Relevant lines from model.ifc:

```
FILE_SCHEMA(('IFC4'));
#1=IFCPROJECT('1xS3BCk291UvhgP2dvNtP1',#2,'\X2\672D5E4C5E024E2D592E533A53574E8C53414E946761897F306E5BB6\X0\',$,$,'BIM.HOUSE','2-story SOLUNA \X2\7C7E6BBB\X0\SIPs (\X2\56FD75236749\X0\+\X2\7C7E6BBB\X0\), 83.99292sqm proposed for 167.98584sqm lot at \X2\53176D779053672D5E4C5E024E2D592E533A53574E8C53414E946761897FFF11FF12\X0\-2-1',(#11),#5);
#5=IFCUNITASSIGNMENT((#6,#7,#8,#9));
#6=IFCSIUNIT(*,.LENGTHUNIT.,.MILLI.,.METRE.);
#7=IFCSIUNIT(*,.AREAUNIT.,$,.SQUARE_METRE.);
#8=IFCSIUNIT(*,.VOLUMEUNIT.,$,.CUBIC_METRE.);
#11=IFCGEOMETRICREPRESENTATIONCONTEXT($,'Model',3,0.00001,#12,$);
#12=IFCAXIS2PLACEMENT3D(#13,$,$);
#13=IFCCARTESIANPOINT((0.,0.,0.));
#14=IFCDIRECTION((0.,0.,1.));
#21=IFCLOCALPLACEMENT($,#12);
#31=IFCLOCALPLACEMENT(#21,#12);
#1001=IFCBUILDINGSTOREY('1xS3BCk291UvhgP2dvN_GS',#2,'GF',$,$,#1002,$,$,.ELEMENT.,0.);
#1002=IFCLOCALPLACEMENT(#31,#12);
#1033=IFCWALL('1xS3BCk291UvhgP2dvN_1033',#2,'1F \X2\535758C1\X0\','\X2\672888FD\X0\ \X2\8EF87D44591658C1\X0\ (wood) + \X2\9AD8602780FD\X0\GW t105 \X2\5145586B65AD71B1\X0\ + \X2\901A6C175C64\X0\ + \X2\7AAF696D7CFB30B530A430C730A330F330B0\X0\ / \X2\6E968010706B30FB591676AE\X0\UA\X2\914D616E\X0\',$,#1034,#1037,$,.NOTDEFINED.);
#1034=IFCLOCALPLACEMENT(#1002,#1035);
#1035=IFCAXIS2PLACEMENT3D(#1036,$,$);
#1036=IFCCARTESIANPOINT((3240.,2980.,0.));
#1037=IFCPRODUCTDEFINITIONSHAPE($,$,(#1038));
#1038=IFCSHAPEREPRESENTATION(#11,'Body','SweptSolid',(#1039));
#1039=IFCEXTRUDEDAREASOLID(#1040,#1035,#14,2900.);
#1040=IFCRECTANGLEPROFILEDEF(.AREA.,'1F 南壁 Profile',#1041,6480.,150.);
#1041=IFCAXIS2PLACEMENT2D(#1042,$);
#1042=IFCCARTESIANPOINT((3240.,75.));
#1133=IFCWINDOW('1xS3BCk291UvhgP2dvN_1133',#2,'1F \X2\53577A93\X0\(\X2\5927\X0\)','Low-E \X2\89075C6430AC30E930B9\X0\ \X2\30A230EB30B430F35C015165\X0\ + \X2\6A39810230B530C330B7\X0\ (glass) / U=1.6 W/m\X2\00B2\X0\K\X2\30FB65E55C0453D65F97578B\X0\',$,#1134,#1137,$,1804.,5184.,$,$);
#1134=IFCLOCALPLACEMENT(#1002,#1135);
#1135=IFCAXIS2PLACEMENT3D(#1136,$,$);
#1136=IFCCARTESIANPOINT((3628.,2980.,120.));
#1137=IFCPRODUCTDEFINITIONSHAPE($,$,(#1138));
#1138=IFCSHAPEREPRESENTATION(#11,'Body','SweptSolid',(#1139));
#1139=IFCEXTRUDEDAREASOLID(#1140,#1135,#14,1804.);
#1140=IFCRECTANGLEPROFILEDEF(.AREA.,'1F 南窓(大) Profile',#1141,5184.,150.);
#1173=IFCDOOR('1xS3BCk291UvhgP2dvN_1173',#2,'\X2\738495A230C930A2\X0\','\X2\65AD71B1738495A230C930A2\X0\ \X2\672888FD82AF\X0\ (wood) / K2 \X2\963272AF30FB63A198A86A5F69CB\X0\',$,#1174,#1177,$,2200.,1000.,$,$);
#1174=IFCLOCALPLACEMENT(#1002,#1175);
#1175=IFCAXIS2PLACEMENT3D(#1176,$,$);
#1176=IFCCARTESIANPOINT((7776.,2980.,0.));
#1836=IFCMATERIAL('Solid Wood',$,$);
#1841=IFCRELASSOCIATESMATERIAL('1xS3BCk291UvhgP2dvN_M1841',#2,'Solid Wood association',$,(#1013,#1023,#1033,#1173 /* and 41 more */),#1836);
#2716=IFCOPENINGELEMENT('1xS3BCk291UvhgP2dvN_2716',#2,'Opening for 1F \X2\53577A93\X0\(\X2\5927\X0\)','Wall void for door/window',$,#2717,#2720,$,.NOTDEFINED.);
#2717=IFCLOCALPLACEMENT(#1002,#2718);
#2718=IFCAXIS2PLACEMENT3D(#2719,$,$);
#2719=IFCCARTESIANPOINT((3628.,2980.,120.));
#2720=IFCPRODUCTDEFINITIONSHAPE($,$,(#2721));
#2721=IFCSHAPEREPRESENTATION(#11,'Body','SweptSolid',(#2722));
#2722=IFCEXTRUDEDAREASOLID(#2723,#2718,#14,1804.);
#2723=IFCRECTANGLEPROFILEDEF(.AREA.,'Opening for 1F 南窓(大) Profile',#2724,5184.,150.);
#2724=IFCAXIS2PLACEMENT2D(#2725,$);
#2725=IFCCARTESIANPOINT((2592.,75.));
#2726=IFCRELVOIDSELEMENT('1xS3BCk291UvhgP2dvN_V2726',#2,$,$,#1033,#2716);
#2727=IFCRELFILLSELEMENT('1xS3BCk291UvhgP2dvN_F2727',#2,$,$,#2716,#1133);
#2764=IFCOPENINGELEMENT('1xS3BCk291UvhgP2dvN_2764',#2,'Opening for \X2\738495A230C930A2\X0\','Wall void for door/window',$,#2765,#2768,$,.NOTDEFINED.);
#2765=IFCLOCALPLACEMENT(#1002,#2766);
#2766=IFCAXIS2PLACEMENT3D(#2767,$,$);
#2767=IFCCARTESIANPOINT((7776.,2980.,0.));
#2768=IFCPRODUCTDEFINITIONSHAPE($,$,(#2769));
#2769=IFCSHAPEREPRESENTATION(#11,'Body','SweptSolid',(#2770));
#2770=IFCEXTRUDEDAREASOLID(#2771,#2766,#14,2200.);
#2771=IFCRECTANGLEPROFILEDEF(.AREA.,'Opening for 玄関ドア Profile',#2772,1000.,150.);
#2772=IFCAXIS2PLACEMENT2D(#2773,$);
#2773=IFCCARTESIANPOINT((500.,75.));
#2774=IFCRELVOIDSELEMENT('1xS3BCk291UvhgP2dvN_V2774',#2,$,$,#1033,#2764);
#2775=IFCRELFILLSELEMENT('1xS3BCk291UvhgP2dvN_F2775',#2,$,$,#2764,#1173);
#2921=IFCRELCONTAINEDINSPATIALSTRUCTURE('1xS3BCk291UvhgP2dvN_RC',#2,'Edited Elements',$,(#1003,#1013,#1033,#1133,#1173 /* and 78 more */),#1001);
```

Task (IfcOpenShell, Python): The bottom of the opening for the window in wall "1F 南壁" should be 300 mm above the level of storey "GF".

```python
import numpy as np
import ifcopenshell
import ifcopenshell.api.geometry
import ifcopenshell.geom
import ifcopenshell.util.element
import ifcopenshell.util.placement
import ifcopenshell.util.shape
import ifcopenshell.util.unit

model = ifcopenshell.open("model.ifc")
unit_scale = ifcopenshell.util.unit.calculate_unit_scale(model)

window = model.by_guid("1xS3BCk291UvhgP2dvN_1133")
opening = window.FillsVoids[0].RelatingOpeningElement
storey = ifcopenshell.util.element.get_container(window, ifc_class="IfcBuildingStorey")
level = ifcopenshell.util.placement.get_local_placement(storey.ObjectPlacement)[2, 3]

# The opening's origin need not be at the sill, so measure its lowest point.
shape = ifcopenshell.geom.create_shape(ifcopenshell.geom.settings(), opening)
bottom = ifcopenshell.util.shape.get_shape_bottom_elevation(shape, shape.geometry) / unit_scale
dz = level + 0.3 / unit_scale - bottom

shift = np.array([0.0, 0.0, dz])
# The window is not placed relative to its opening, so move both.
for product in (opening, window):
    matrix = ifcopenshell.util.placement.get_local_placement(product.ObjectPlacement)
    matrix[:3, 3] += shift
    ifcopenshell.api.geometry.edit_object_placement(model, product=product, matrix=matrix, is_si=False)

print(f"moved by {dz * unit_scale:+.3f} m")

model.write("model_edited.ifc")
```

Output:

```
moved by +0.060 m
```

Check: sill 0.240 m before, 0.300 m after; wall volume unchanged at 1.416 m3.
